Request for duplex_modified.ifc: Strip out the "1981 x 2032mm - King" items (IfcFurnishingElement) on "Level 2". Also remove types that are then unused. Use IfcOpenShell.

First a look at what the model holds.

```python
import ifcopenshell
import ifcopenshell.util.element

model = ifcopenshell.open("duplex_modified.ifc")
print(model.schema)
storey = next(s for s in model.by_type("IfcBuildingStorey") if s.Name == "Level 2")
furniture = [e for e in ifcopenshell.util.element.get_decomposition(storey) if e.is_a("IfcFurnishingElement")]
seen = {}
for e in furniture:
    element_type = ifcopenshell.util.element.get_type(e)
    name = element_type.Name if element_type not in (None, e) else None
    seen[name] = seen.get(name, 0) + 1
for name, count in sorted(seen.items(), key=str):
    print(count, "x", name)
```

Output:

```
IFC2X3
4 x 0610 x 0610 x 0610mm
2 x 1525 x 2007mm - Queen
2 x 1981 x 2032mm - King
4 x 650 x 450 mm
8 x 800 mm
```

```python
import ifcopenshell
import ifcopenshell.api.root
import ifcopenshell.util.element

model = ifcopenshell.open("duplex_modified.ifc")

storey = next(s for s in model.by_type("IfcBuildingStorey") if s.Name == "Level 2")
furniture = [e for e in ifcopenshell.util.element.get_decomposition(storey) if e.is_a("IfcFurnishingElement")]
targets = [e for e in furniture if (t := ifcopenshell.util.element.get_type(e)) not in (None, e) and t.Name == "1981 x 2032mm - King"]
types = {ifcopenshell.util.element.get_type(e) for e in targets} - {None, *targets}

for e in targets:
    ifcopenshell.api.root.remove_product(model, product=e)
print(len(targets), "removed")

unused = [t for t in types if not ifcopenshell.util.element.get_types(t)]
for t in unused:
    ifcopenshell.api.root.remove_product(model, product=t)
print(len(unused), "unused types removed")

model.write("duplex_modified_rev.ifc")
```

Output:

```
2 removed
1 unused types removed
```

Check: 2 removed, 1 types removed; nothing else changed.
